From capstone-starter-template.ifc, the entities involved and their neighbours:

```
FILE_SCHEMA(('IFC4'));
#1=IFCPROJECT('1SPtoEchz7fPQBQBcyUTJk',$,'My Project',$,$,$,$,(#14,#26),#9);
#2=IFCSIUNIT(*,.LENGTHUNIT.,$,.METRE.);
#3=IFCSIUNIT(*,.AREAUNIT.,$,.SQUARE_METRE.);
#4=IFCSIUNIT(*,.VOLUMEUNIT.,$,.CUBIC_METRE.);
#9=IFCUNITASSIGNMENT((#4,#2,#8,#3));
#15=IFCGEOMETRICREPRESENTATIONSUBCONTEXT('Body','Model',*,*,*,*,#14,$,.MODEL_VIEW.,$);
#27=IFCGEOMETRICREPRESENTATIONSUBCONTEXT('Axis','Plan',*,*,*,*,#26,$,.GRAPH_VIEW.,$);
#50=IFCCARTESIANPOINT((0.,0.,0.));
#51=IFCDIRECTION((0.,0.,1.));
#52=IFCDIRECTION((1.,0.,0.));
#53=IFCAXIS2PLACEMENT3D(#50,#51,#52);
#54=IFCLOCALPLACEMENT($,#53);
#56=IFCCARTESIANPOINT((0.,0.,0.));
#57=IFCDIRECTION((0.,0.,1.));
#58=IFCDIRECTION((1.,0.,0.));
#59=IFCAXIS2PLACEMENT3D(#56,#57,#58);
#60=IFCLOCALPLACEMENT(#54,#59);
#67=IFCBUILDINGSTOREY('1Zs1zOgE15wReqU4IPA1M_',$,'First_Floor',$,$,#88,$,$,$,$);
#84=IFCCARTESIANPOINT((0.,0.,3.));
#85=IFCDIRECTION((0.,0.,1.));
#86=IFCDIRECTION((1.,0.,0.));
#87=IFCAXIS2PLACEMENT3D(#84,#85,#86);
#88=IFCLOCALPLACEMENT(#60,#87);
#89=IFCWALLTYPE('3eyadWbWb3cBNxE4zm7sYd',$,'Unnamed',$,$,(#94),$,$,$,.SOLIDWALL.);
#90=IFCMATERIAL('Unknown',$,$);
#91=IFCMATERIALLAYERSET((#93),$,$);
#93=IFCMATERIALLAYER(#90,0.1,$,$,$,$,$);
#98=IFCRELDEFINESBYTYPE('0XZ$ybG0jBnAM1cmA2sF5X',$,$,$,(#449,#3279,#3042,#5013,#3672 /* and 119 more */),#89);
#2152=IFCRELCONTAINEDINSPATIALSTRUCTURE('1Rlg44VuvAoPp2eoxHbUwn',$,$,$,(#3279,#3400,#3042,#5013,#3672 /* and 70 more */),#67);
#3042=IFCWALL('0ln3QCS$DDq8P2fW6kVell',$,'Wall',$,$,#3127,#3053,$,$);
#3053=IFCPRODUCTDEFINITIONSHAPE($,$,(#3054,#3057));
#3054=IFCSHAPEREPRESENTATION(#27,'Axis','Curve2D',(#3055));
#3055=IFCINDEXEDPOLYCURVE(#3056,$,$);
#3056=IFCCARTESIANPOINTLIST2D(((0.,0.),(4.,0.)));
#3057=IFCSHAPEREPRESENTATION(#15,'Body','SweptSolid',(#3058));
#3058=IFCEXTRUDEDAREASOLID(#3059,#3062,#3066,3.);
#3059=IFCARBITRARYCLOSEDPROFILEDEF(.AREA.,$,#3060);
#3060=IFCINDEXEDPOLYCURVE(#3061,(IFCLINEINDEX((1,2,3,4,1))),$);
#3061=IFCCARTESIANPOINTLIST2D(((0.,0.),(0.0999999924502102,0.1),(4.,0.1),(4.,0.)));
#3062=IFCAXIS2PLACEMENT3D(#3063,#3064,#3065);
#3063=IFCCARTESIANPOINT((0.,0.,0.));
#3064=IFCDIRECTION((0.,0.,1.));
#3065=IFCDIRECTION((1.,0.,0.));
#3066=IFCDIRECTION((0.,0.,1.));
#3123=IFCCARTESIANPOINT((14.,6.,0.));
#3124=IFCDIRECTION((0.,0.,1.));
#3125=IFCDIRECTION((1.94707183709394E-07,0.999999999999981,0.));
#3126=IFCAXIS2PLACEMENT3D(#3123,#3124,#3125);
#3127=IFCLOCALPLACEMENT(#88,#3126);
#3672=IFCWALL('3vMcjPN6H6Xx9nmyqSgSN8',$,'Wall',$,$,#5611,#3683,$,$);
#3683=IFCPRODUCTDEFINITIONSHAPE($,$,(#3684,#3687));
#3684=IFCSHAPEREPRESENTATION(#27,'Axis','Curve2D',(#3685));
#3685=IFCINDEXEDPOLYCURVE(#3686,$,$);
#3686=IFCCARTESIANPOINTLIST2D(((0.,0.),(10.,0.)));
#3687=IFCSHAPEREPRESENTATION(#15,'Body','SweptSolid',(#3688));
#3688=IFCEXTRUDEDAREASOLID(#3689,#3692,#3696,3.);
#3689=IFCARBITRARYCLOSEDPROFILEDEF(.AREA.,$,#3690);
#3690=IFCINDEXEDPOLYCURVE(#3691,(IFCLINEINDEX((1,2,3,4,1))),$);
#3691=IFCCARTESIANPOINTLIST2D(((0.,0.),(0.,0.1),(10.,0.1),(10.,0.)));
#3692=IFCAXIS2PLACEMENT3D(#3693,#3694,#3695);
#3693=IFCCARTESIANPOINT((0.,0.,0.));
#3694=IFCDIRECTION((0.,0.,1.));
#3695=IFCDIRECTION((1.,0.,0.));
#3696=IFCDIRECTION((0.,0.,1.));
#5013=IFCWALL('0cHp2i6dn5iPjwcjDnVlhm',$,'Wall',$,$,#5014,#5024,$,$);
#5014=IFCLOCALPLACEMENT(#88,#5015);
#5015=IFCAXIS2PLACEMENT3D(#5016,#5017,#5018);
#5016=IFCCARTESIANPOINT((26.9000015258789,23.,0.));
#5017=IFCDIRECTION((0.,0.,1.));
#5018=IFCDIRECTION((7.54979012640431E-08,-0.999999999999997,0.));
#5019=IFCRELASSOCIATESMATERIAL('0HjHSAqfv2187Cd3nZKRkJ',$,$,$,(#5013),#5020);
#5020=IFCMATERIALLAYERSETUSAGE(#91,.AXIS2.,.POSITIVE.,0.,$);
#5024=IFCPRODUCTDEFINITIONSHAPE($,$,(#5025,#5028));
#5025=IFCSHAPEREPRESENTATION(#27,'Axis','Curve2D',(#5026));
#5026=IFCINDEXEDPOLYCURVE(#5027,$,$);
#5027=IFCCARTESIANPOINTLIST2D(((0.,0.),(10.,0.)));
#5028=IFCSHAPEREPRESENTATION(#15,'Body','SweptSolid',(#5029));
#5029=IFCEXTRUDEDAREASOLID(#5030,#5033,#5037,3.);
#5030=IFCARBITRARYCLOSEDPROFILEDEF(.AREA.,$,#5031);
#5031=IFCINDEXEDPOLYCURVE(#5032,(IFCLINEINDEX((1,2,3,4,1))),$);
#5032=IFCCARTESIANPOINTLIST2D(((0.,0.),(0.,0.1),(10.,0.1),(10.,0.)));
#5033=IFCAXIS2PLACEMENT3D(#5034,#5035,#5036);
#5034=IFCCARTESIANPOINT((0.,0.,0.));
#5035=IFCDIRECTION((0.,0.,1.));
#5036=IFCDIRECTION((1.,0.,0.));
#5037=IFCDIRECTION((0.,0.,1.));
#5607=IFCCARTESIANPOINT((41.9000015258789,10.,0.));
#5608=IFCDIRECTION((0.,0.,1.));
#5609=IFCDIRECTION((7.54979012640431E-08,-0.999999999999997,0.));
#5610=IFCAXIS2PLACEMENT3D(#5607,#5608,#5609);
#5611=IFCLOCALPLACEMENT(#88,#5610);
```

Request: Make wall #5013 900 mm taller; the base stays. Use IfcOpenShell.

```python
import ifcopenshell
import ifcopenshell.geom
import ifcopenshell.util.representation
import ifcopenshell.util.shape
import ifcopenshell.util.unit

model = ifcopenshell.open("capstone-starter-template.ifc")
unit_scale = ifcopenshell.util.unit.calculate_unit_scale(model)
settings = ifcopenshell.geom.settings()


def volume(element):
    """Net volume in cubic metres, openings subtracted."""
    shape = ifcopenshell.geom.create_shape(settings, element)
    return ifcopenshell.util.shape.get_volume(shape.geometry)


wall = model.by_guid("0cHp2i6dn5iPjwcjDnVlhm")
before = volume(wall)

body = ifcopenshell.util.representation.get_representation(wall, "Model", "Body")
solid = body.Items[0]
old_height = solid.Depth
solid.Depth += 0.9 / unit_scale
after = volume(wall)

print(f"height {old_height:g} -> {solid.Depth:g}, volume {before:.3f} -> {after:.3f} m3")

model.write("capstone-starter-template_v2.ifc")
```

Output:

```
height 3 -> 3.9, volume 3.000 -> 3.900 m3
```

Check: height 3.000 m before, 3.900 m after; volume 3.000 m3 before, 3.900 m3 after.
